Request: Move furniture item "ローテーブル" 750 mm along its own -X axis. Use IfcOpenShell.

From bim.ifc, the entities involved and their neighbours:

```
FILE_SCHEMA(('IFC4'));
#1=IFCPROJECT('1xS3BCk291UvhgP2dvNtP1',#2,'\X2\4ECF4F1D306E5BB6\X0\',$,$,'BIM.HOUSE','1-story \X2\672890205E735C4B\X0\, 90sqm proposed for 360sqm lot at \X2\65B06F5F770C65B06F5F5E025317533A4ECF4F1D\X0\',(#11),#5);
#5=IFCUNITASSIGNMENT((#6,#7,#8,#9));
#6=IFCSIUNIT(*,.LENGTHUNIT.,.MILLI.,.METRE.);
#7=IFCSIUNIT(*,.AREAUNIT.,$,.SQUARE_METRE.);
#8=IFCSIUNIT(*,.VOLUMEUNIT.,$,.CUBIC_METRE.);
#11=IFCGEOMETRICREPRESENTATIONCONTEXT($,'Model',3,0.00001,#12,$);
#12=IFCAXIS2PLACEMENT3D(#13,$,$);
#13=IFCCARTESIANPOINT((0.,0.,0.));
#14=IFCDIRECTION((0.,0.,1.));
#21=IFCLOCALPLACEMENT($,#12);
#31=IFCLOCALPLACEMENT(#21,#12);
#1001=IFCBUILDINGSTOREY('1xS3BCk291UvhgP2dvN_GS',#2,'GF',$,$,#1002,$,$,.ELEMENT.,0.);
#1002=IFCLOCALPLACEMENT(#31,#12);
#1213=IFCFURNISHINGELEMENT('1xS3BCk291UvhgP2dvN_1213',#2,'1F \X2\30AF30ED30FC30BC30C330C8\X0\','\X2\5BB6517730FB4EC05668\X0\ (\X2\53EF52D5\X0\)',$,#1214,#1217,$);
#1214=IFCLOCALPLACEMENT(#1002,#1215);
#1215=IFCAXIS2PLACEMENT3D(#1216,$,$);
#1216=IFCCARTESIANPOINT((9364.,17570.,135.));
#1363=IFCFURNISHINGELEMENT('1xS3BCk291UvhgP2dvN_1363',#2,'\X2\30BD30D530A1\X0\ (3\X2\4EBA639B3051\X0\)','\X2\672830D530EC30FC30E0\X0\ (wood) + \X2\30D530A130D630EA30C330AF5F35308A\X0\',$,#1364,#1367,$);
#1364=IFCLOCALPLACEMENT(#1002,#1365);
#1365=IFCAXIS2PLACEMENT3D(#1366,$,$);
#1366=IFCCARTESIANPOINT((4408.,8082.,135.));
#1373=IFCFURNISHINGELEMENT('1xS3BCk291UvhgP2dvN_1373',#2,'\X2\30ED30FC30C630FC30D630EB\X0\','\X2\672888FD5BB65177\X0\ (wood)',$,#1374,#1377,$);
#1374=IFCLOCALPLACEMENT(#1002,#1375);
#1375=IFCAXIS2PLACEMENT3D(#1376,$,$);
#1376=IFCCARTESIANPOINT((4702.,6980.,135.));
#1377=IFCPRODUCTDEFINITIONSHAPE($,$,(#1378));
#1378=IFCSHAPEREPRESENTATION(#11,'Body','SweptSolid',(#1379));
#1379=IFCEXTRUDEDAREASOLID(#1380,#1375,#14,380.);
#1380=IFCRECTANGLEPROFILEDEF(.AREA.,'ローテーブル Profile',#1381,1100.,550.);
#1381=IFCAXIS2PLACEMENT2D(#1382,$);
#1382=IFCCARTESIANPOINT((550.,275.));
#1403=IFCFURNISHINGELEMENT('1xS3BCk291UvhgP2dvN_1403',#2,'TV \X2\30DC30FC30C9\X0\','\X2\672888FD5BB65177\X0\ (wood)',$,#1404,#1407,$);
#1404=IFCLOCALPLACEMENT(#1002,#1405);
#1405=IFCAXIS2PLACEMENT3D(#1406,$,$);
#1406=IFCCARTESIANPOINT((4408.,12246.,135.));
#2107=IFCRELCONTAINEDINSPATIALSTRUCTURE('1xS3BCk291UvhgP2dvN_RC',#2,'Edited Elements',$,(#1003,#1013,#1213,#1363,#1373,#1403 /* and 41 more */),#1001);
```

```python
import ifcopenshell
import ifcopenshell.api.geometry
import ifcopenshell.util.placement

model = ifcopenshell.open("bim.ifc")

item = model.by_guid("1xS3BCk291UvhgP2dvN_1373")
matrix = ifcopenshell.util.placement.get_local_placement(item.ObjectPlacement)
matrix[:3, 3] -= matrix[:3, 0] * 750.0
ifcopenshell.api.geometry.edit_object_placement(model, product=item, matrix=matrix, is_si=False)

print(ifcopenshell.util.placement.get_local_placement(item.ObjectPlacement).round(3) + 0.0)

model.write("bim_edited.ifc")
```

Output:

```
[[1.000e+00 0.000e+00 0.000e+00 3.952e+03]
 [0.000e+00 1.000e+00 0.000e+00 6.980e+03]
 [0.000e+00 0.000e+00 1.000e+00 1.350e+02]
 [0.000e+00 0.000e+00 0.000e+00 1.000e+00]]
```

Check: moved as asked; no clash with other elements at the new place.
